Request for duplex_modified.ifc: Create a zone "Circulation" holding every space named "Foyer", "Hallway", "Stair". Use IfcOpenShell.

First a look at what the model holds.

```python
import ifcopenshell

model = ifcopenshell.open("duplex_modified.ifc")
print(model.schema)
seen = {}
for space in model.by_type("IfcSpace"):
    seen[space.LongName] = seen.get(space.LongName, 0) + 1
for name, count in sorted(seen.items(), key=str):
    print(count, "x", name)
print("zones:", [z.Name for z in model.by_type("IfcZone")][:20])
```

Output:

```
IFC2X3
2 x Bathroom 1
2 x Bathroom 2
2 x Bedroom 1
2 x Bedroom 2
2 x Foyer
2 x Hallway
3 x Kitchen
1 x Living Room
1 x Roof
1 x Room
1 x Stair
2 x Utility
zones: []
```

```python
import ifcopenshell
import ifcopenshell.api.group
import ifcopenshell.api.root

model = ifcopenshell.open("duplex_modified.ifc")

names = {"Foyer", "Hallway", "Stair"}
spaces = [s for s in model.by_type("IfcSpace") if s.LongName in names]

zone = ifcopenshell.api.root.create_entity(model, ifc_class="IfcZone", name="Circulation")
ifcopenshell.api.group.assign_group(model, products=spaces, group=zone)
print(len(spaces), "spaces in", zone.Name)

model.write("duplex_modified_v2.ifc")
```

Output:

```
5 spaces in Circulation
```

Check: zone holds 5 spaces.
